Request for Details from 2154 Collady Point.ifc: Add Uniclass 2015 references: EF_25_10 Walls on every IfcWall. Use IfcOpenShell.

First a look at what the model holds.

```python
import ifcopenshell

model = ifcopenshell.open("Details from 2154 Collady Point.ifc")
print(model.schema)
print("classifications:", [c.Name for c in model.by_type("IfcClassification")])
for ifc_class in ("IfcDoor", "IfcRoof", "IfcStair", "IfcWall", "IfcWindow"):
    print(ifc_class, len(model.by_type(ifc_class)))
```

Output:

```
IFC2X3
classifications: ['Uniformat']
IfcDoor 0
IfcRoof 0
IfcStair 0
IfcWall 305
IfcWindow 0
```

```python
import ifcopenshell
import ifcopenshell.api.classification

model = ifcopenshell.open("Details from 2154 Collady Point.ifc")

# IFC2X3 requires Source and Edition and has no link from the project to the system.
system = model.create_entity("IfcClassification", Source="NBS", Edition="2015", Name="Uniclass 2015")

codes = {
    "IfcWall": ("EF_25_10", "Walls"),
}
for ifc_class, (code, name) in codes.items():
    products = model.by_type(ifc_class)
    ifcopenshell.api.classification.add_reference(
        model, products=products, classification=system, identification=code, name=name
    )
    print(code, len(products))

model.write("Details from 2154 Collady Point_updated.ifc")
```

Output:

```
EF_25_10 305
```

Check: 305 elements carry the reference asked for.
